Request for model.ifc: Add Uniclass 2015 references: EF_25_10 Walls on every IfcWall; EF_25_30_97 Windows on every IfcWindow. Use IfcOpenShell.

First a look at what the model holds.

```python
import ifcopenshell

model = ifcopenshell.open("model.ifc")
print(model.schema)
print("classifications:", [c.Name for c in model.by_type("IfcClassification")])
for ifc_class in ("IfcDoor", "IfcRoof", "IfcStair", "IfcWall", "IfcWindow"):
    print(ifc_class, len(model.by_type(ifc_class)))
```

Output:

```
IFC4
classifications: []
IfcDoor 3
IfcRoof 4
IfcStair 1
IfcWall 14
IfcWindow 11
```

```python
import ifcopenshell
import ifcopenshell.api.classification

model = ifcopenshell.open("model.ifc")

system = ifcopenshell.api.classification.add_classification(model, classification="Uniclass 2015")

codes = {
    "IfcWall": ("EF_25_10", "Walls"),
    "IfcWindow": ("EF_25_30_97", "Windows"),
}
for ifc_class, (code, name) in codes.items():
    products = model.by_type(ifc_class)
    ifcopenshell.api.classification.add_reference(
        model, products=products, classification=system, identification=code, name=name
    )
    print(code, len(products))

model.write("model_edited.ifc")
```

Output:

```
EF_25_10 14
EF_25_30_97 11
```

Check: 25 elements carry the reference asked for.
